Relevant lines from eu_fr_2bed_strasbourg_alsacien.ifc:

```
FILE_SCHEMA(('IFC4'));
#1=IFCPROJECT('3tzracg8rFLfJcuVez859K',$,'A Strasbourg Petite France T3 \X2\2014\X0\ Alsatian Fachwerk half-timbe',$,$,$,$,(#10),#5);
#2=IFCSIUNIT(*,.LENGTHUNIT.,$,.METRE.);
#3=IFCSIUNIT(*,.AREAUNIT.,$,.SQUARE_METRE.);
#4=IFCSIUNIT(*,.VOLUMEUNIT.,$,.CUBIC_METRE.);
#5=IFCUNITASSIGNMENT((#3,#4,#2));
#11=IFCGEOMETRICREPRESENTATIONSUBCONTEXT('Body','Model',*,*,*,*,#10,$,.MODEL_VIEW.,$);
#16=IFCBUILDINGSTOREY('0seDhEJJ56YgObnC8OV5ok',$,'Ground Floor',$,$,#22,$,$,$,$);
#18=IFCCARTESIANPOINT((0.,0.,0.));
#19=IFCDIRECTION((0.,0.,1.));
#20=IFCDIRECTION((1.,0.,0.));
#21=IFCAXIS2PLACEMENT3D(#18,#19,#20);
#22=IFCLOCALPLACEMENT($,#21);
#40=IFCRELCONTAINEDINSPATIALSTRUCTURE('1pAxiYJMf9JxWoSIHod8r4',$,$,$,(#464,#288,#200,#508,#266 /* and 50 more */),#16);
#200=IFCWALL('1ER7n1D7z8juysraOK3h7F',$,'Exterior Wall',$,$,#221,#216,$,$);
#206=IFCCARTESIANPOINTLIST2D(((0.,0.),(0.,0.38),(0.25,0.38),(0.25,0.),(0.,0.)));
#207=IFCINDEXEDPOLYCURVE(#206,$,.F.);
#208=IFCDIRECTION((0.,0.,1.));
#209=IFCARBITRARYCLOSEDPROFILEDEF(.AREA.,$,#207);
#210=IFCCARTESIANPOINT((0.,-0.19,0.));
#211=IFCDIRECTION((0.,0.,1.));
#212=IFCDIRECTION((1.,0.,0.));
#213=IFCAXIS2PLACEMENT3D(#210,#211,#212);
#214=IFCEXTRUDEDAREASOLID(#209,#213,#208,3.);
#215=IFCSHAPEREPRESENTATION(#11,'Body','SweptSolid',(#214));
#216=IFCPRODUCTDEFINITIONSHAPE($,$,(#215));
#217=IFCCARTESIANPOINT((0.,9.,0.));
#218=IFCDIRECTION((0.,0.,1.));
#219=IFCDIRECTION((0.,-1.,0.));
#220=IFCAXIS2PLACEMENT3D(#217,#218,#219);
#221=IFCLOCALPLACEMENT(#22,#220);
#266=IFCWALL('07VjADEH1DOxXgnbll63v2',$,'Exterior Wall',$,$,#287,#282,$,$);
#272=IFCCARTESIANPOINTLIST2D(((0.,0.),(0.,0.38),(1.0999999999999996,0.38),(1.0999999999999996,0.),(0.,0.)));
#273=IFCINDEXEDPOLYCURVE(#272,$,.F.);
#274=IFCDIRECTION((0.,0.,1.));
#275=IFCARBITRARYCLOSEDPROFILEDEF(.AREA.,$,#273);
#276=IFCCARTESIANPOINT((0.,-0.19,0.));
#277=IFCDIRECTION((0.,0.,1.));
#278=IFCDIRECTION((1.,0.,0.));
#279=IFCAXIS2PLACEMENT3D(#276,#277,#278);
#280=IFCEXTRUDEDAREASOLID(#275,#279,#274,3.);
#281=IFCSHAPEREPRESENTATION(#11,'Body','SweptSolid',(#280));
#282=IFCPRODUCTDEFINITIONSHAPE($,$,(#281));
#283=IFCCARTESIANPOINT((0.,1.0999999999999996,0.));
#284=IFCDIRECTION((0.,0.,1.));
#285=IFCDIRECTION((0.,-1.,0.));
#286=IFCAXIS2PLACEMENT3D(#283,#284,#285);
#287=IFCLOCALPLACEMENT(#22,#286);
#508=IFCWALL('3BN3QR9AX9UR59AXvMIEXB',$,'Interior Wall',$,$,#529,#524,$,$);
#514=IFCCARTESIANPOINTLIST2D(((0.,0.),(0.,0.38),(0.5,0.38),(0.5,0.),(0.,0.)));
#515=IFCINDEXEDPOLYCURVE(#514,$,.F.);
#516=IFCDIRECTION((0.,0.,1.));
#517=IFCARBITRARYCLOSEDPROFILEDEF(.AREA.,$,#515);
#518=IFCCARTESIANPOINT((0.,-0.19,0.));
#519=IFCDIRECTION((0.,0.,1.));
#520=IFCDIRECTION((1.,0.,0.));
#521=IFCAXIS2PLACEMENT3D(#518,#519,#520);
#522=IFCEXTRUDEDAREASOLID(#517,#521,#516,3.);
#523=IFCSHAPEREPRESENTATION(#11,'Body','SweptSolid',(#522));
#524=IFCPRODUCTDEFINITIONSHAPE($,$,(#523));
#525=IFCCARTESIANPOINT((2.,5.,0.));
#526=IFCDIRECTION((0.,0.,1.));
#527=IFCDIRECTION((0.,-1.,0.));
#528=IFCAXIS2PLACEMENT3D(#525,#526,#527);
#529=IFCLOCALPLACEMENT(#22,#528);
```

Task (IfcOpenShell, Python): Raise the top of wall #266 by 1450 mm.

```python
import ifcopenshell
import ifcopenshell.geom
import ifcopenshell.util.representation
import ifcopenshell.util.shape
import ifcopenshell.util.unit

model = ifcopenshell.open("eu_fr_2bed_strasbourg_alsacien.ifc")
unit_scale = ifcopenshell.util.unit.calculate_unit_scale(model)
settings = ifcopenshell.geom.settings()


def volume(element):
    """Net volume in cubic metres, openings subtracted."""
    shape = ifcopenshell.geom.create_shape(settings, element)
    return ifcopenshell.util.shape.get_volume(shape.geometry)


wall = model.by_guid("07VjADEH1DOxXgnbll63v2")
before = volume(wall)

body = ifcopenshell.util.representation.get_representation(wall, "Model", "Body")
solid = body.Items[0]
old_height = solid.Depth
solid.Depth += 1.45 / unit_scale
after = volume(wall)

print(f"height {old_height:g} -> {solid.Depth:g}, volume {before:.3f} -> {after:.3f} m3")

model.write("eu_fr_2bed_strasbourg_alsacien-out.ifc")
```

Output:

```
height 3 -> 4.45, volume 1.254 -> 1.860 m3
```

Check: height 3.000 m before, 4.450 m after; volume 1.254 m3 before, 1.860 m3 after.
